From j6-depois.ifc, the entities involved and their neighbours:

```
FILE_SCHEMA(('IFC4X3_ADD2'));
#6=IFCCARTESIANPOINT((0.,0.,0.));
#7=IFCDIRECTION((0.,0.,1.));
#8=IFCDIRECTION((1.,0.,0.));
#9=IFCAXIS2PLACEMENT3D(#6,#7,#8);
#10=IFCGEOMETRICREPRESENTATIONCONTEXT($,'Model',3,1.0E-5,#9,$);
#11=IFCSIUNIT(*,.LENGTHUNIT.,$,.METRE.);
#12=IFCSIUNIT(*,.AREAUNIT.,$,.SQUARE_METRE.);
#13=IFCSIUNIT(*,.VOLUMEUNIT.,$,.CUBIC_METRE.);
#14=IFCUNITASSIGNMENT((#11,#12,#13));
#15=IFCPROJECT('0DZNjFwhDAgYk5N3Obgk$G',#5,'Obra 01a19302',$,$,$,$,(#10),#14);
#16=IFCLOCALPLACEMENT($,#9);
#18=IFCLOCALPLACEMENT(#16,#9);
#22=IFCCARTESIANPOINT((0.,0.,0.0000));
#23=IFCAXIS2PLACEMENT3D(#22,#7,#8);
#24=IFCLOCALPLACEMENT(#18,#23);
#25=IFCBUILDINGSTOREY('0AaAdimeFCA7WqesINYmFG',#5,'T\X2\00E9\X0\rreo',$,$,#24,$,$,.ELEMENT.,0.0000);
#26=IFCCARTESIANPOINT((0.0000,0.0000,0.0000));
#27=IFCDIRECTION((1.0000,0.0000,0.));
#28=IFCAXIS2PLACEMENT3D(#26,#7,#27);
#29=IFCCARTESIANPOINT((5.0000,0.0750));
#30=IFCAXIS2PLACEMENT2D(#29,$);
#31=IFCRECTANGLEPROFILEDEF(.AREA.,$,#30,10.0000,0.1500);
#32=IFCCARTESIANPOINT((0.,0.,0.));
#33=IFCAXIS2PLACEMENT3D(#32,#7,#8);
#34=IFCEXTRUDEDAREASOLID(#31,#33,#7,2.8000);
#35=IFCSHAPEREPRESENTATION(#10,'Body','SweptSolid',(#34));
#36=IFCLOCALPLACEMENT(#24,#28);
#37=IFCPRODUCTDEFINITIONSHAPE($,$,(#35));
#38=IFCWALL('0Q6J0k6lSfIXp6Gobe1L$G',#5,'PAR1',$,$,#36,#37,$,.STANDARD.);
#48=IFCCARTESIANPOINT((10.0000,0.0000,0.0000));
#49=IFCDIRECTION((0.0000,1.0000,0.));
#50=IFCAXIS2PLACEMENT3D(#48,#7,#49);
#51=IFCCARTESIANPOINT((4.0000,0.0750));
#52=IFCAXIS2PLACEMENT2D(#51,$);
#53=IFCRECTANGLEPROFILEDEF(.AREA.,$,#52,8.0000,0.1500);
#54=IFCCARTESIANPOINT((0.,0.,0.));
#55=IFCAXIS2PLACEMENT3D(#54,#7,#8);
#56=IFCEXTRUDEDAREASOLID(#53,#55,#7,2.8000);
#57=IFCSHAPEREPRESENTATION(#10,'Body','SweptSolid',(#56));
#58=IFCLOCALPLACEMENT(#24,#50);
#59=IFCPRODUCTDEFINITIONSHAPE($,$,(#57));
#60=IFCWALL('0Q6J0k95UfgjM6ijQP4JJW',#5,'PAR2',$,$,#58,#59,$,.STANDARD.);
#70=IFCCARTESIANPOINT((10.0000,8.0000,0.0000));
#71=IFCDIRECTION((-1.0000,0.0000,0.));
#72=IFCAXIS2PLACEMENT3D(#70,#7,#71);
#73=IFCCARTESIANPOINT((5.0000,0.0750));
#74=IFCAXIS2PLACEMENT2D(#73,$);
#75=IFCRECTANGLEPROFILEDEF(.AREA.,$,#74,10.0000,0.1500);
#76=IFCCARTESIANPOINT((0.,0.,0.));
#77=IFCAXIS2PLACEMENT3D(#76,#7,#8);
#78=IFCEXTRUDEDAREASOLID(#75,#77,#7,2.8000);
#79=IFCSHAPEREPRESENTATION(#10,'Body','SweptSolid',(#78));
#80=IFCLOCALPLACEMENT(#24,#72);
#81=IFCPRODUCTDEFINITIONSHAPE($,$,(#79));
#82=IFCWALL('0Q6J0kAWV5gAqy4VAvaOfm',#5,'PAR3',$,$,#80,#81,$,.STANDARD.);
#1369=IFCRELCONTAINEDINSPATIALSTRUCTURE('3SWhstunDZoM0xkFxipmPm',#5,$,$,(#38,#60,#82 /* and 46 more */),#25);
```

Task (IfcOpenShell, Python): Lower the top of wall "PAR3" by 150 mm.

```python
import ifcopenshell
import ifcopenshell.geom
import ifcopenshell.util.shape
import ifcopenshell.util.unit

model = ifcopenshell.open("j6-depois.ifc")
unit_scale = ifcopenshell.util.unit.calculate_unit_scale(model)
settings = ifcopenshell.geom.settings()


def volume(element):
    """Net volume in cubic metres, openings subtracted."""
    shape = ifcopenshell.geom.create_shape(settings, element)
    return ifcopenshell.util.shape.get_volume(shape.geometry)


wall = model.by_guid("0Q6J0kAWV5gAqy4VAvaOfm")
before = volume(wall)

body = next(r for r in wall.Representation.Representations if r.RepresentationIdentifier == "Body")
solid = body.Items[0]
old_height = solid.Depth
solid.Depth -= 0.15 / unit_scale
after = volume(wall)

print(f"height {old_height:g} -> {solid.Depth:g}, volume {before:.3f} -> {after:.3f} m3")

model.write("j6-depois_rev.ifc")
```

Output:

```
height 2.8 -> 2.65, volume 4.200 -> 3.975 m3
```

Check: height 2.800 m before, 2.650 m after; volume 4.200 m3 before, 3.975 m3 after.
